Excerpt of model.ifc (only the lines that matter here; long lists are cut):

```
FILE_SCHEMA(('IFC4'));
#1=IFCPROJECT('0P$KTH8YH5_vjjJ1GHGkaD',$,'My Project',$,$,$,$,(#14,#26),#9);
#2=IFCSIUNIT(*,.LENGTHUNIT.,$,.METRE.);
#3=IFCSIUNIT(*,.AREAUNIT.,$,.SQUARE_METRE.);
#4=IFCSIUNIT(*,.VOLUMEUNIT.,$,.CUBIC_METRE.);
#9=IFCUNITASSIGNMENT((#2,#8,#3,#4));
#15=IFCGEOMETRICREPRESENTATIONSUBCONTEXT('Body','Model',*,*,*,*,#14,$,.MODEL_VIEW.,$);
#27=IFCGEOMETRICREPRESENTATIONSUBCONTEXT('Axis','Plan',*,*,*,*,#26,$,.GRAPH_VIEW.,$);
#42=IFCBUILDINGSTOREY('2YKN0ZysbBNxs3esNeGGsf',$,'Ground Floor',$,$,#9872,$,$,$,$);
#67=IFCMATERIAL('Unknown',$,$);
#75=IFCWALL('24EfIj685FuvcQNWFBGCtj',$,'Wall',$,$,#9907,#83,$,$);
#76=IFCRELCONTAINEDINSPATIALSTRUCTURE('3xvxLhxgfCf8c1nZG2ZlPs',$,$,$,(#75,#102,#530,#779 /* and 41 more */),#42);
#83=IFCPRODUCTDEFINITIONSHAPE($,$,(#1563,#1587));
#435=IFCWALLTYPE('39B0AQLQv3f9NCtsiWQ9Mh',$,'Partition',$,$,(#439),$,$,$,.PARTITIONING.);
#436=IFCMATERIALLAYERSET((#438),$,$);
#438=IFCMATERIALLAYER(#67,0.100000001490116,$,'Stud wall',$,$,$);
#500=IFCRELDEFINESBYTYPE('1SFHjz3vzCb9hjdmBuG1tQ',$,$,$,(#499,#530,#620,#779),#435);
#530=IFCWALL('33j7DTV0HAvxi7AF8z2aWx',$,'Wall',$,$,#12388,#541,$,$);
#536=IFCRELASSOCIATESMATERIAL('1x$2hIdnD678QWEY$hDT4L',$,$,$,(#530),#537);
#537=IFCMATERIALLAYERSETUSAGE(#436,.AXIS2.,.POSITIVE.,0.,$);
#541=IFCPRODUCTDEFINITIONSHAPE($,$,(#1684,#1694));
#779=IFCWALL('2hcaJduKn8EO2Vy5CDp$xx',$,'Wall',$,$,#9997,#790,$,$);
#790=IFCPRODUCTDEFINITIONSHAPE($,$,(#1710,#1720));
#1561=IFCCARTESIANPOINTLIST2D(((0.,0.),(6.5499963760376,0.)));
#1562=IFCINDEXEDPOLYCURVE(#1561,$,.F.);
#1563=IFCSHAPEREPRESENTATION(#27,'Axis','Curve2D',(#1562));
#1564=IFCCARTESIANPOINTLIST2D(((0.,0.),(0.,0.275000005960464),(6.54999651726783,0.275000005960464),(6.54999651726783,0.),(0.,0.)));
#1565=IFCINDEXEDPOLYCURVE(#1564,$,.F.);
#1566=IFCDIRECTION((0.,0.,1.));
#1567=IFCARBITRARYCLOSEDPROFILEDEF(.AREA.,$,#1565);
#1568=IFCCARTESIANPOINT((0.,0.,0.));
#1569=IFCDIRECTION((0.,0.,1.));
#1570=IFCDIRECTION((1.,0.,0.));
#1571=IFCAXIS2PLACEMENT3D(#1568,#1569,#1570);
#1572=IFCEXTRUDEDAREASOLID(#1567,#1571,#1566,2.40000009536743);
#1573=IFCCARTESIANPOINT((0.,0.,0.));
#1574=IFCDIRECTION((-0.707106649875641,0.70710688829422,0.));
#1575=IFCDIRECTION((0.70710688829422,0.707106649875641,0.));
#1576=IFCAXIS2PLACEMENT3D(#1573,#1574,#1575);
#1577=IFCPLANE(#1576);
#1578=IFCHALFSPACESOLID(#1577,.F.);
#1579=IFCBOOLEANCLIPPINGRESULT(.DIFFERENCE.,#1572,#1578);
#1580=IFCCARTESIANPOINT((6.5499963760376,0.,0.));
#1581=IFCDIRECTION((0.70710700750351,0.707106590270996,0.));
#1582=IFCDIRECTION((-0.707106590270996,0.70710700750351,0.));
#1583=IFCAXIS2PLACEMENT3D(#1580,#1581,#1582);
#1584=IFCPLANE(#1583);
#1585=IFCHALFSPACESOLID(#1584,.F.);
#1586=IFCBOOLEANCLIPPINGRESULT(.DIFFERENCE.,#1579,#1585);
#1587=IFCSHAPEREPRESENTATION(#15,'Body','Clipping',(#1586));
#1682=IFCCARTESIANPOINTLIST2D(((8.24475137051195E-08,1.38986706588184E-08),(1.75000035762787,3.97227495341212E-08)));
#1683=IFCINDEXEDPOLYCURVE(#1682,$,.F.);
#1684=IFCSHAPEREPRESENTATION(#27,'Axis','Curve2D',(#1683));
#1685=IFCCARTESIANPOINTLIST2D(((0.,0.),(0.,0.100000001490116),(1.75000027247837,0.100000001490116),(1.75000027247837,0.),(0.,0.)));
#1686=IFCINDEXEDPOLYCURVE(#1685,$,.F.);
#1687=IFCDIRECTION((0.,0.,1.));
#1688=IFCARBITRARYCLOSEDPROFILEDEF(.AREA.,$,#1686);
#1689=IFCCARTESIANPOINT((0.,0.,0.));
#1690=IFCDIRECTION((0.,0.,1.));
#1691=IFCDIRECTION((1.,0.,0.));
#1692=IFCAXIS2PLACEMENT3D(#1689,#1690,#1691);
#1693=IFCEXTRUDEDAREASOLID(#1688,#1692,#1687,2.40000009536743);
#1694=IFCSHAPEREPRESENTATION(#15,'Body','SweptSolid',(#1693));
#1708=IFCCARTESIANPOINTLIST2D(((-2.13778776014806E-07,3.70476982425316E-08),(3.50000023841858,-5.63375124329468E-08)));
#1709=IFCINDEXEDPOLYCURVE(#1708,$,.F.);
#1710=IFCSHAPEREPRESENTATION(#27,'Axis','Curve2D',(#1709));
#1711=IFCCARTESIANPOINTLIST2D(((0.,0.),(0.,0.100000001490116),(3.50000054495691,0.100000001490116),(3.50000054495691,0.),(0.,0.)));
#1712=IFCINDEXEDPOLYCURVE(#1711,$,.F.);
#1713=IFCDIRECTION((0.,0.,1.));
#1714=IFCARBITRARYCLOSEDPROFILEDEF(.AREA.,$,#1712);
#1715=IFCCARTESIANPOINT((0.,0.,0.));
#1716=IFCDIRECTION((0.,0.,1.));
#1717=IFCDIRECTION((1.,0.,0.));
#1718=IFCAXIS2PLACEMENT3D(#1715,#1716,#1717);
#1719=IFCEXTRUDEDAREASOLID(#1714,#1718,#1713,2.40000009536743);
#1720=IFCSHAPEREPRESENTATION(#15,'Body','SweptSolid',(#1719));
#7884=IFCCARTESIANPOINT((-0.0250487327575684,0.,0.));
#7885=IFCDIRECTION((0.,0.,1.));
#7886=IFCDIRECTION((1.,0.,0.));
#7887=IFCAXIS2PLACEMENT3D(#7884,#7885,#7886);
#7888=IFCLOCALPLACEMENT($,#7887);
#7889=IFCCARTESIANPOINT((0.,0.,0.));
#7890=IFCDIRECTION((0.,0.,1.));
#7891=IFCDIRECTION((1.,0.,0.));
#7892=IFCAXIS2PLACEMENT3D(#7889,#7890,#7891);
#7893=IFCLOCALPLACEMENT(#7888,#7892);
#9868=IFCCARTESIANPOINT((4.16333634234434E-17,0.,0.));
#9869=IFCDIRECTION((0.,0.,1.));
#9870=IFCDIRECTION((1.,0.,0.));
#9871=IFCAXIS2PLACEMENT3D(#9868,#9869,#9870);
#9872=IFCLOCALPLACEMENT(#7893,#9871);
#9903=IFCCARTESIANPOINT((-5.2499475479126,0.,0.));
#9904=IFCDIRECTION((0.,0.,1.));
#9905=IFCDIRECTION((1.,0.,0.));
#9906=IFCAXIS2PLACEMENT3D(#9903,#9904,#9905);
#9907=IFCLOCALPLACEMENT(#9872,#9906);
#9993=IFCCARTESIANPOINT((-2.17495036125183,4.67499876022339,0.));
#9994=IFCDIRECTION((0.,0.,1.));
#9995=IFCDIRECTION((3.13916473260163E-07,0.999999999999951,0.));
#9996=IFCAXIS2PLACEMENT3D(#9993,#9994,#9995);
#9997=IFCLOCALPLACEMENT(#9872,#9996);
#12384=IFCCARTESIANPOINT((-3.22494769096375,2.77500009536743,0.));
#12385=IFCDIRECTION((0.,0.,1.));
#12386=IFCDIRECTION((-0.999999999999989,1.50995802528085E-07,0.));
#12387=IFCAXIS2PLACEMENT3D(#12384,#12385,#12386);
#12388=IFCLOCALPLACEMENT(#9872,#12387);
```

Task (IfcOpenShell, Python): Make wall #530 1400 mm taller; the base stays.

```python
import ifcopenshell
import ifcopenshell.geom
import ifcopenshell.util.representation
import ifcopenshell.util.shape
import ifcopenshell.util.unit

model = ifcopenshell.open("model.ifc")
unit_scale = ifcopenshell.util.unit.calculate_unit_scale(model)
settings = ifcopenshell.geom.settings()


def volume(element):
    """Net volume in cubic metres, openings subtracted."""
    shape = ifcopenshell.geom.create_shape(settings, element)
    return ifcopenshell.util.shape.get_volume(shape.geometry)


wall = model.by_guid("33j7DTV0HAvxi7AF8z2aWx")
before = volume(wall)

body = ifcopenshell.util.representation.get_representation(wall, "Model", "Body")
solid = body.Items[0]
old_height = solid.Depth
solid.Depth += 1.4 / unit_scale
after = volume(wall)

print(f"height {old_height:g} -> {solid.Depth:g}, volume {before:.3f} -> {after:.3f} m3")

model.write("model-out.ifc")
```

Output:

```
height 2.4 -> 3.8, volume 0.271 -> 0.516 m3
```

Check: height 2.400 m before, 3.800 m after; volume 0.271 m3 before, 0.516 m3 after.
